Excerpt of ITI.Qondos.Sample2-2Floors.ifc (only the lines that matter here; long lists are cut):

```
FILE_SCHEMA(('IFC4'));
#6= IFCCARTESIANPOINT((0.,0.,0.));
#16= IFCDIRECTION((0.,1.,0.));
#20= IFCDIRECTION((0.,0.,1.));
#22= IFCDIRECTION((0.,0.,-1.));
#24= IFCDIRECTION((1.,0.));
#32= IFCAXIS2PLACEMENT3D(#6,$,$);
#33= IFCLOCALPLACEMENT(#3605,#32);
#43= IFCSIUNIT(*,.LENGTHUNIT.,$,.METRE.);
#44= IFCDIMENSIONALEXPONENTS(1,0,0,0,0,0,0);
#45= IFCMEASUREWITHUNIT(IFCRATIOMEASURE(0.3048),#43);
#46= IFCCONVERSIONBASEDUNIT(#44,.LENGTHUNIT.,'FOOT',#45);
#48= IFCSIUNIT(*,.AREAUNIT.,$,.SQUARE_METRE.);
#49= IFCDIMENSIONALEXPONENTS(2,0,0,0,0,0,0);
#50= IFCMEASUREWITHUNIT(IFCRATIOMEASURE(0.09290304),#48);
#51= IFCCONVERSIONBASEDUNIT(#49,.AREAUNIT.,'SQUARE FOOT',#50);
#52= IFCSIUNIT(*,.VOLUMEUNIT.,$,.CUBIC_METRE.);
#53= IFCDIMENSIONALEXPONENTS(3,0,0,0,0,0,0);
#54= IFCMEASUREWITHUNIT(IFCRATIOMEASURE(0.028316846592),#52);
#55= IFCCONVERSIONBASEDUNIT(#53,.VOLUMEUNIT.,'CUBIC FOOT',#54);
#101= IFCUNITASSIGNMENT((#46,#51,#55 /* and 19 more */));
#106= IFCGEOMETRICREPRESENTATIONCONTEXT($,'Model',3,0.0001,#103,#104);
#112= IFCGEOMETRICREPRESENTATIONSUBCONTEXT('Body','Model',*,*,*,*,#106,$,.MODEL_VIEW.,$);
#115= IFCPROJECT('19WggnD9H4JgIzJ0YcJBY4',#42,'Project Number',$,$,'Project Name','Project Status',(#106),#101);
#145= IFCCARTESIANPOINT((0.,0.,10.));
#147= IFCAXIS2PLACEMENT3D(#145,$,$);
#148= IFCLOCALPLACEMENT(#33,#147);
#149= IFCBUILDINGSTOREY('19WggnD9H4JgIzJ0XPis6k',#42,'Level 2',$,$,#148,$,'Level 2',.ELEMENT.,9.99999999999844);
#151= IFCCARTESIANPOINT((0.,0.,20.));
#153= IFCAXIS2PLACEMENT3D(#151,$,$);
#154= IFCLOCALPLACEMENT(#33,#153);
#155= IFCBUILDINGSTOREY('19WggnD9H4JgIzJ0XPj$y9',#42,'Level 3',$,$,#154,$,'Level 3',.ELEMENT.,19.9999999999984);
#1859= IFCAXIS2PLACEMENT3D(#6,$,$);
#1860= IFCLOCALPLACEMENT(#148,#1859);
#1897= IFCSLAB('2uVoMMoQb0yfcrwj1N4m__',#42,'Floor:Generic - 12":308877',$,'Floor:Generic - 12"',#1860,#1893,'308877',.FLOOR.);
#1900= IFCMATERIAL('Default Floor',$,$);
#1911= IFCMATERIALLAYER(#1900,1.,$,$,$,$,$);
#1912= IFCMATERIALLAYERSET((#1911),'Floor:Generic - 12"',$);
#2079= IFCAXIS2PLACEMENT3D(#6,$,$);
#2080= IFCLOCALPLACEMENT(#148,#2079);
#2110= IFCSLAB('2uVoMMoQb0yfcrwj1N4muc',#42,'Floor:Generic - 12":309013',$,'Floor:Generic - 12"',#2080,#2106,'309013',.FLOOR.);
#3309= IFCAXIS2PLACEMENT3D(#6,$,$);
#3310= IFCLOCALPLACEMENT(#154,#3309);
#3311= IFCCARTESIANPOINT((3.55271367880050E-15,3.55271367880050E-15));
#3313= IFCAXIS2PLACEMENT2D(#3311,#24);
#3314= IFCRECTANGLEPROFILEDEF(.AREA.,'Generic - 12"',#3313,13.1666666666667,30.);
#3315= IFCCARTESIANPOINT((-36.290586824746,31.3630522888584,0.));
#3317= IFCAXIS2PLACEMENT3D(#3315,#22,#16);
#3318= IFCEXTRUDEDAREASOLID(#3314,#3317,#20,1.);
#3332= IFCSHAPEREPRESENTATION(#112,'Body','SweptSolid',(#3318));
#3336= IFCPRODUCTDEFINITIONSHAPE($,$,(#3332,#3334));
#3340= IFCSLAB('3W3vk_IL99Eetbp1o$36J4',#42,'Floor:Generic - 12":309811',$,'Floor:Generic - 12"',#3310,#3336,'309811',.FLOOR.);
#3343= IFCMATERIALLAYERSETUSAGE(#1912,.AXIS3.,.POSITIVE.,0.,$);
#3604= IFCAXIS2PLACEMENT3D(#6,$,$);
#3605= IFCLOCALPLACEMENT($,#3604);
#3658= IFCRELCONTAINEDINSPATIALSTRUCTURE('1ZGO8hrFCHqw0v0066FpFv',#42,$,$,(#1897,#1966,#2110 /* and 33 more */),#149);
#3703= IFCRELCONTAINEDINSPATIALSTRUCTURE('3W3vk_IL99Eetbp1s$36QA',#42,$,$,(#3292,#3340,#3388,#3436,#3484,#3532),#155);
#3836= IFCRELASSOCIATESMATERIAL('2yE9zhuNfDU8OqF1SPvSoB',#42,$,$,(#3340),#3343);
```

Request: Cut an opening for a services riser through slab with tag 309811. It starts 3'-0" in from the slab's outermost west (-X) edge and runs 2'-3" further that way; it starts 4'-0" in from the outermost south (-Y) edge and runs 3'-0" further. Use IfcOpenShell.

```python
import numpy as np
import ifcopenshell
import ifcopenshell.api.feature
import ifcopenshell.api.geometry
import ifcopenshell.api.root
import ifcopenshell.geom
import ifcopenshell.util.placement
import ifcopenshell.util.representation
import ifcopenshell.util.shape
import ifcopenshell.util.unit

model = ifcopenshell.open("ITI.Qondos.Sample2-2Floors.ifc")
unit_scale = ifcopenshell.util.unit.calculate_unit_scale(model)
settings = ifcopenshell.geom.settings()


def volume(element):
    """Net volume in cubic metres, openings subtracted."""
    shape = ifcopenshell.geom.create_shape(settings, element)
    return ifcopenshell.util.shape.get_volume(shape.geometry)


slab = model.by_guid("3W3vk_IL99Eetbp1o$36J4")
before = volume(slab)

# Extent in the slab's own axes, in metres. The edges named are its -X and -Y sides.
slab_shape = ifcopenshell.geom.create_shape(settings, slab)
vertices = ifcopenshell.util.shape.get_vertices(slab_shape.geometry)
x_min, y_min, bottom = vertices.min(axis=0)
top = vertices[:, 2].max()

opening = ifcopenshell.api.root.create_entity(model, ifc_class="IfcOpeningElement", name="Services riser opening", predefined_type="OPENING")
context = ifcopenshell.util.representation.get_context(model, "Model", "Body", "MODEL_VIEW")
width, depth = 0.6858, 0.9144
outline = [(0.0, 0.0), (width, 0.0), (width, depth), (0.0, depth), (0.0, 0.0)]
# Overshoot both faces by 50 mm so the cut is clean.
shape = ifcopenshell.api.geometry.add_slab_representation(
    model, context=context, depth=top - bottom + 0.1, polyline=outline
)
ifcopenshell.api.geometry.assign_representation(model, product=opening, representation=shape)

matrix = ifcopenshell.util.placement.get_local_placement(slab.ObjectPlacement)
matrix[:, 3] = matrix @ np.append(np.array([x_min + 0.9144, y_min + 1.2192, bottom - 0.05]) / unit_scale, 1.0)
ifcopenshell.api.geometry.edit_object_placement(model, product=opening, matrix=matrix, is_si=False)
ifcopenshell.api.feature.add_feature(model, feature=opening, element=slab)

after = volume(slab)

print(f"slab volume {before:.3f} -> {after:.3f} m3")

model.write("ITI.Qondos.Sample2-2Floors_rev.ifc")
```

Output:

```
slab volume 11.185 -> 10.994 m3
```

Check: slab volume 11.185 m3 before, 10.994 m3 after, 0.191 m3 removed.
